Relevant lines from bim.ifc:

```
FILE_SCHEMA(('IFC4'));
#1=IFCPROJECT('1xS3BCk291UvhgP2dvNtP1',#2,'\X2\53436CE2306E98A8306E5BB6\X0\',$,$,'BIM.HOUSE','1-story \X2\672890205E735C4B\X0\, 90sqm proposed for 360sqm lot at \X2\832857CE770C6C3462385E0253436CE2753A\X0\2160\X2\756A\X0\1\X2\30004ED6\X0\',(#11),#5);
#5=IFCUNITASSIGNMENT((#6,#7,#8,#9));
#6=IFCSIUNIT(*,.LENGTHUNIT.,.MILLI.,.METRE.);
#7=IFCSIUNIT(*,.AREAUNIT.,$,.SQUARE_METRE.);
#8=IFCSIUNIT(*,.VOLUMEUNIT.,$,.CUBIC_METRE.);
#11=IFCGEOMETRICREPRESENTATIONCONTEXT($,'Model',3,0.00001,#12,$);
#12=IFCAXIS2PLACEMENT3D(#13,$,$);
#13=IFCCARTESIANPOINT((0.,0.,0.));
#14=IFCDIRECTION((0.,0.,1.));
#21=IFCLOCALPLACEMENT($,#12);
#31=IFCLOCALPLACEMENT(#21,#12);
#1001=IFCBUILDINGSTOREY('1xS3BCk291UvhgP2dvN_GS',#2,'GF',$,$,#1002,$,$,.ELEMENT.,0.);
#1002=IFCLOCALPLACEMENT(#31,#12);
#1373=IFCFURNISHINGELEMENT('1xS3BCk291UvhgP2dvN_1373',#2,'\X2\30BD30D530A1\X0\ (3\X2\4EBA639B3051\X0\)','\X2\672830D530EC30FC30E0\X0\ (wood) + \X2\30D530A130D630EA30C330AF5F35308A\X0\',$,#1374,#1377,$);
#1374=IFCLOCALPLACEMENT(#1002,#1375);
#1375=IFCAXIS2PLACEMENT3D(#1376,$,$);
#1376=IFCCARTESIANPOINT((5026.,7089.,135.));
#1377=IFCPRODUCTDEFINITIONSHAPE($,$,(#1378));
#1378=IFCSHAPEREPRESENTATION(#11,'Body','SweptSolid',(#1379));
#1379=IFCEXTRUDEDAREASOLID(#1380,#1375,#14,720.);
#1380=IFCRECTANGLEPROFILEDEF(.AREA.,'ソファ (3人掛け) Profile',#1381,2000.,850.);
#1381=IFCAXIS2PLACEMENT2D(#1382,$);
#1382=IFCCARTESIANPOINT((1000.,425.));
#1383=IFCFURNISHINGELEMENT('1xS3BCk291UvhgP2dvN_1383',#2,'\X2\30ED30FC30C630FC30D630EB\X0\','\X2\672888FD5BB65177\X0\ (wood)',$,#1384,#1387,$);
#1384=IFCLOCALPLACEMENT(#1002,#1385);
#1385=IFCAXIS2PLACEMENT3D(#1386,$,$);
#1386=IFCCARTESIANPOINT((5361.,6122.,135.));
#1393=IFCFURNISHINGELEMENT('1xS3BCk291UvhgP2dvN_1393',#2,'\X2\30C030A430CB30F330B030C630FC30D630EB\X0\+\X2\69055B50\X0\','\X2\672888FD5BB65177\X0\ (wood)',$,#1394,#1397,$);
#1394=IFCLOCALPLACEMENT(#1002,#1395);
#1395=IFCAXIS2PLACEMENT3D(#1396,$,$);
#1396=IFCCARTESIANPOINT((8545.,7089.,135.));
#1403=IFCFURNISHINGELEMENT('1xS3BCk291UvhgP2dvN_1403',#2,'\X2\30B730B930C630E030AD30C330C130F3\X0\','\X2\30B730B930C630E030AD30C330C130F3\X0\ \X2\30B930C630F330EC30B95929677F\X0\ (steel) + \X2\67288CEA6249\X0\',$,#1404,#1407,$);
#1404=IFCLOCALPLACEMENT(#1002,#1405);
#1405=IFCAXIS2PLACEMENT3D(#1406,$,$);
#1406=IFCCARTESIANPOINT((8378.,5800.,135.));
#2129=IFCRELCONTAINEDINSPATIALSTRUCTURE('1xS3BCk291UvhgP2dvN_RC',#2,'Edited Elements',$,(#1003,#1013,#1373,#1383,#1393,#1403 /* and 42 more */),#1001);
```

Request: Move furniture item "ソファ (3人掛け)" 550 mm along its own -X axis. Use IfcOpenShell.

```python
import ifcopenshell
import ifcopenshell.api.geometry
import ifcopenshell.util.placement
import ifcopenshell.util.unit

model = ifcopenshell.open("bim.ifc")
unit_scale = ifcopenshell.util.unit.calculate_unit_scale(model)

item = model.by_guid("1xS3BCk291UvhgP2dvN_1373")
matrix = ifcopenshell.util.placement.get_local_placement(item.ObjectPlacement)
matrix[:3, 3] -= matrix[:3, 0] * 0.55 / unit_scale
ifcopenshell.api.geometry.edit_object_placement(model, product=item, matrix=matrix, is_si=False)

print(ifcopenshell.util.placement.get_local_placement(item.ObjectPlacement).round(3) + 0.0)

model.write("bim-out.ifc")
```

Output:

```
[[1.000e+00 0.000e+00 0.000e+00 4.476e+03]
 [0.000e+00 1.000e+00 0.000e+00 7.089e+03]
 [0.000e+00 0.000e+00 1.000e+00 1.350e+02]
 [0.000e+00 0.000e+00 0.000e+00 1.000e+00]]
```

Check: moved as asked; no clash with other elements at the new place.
